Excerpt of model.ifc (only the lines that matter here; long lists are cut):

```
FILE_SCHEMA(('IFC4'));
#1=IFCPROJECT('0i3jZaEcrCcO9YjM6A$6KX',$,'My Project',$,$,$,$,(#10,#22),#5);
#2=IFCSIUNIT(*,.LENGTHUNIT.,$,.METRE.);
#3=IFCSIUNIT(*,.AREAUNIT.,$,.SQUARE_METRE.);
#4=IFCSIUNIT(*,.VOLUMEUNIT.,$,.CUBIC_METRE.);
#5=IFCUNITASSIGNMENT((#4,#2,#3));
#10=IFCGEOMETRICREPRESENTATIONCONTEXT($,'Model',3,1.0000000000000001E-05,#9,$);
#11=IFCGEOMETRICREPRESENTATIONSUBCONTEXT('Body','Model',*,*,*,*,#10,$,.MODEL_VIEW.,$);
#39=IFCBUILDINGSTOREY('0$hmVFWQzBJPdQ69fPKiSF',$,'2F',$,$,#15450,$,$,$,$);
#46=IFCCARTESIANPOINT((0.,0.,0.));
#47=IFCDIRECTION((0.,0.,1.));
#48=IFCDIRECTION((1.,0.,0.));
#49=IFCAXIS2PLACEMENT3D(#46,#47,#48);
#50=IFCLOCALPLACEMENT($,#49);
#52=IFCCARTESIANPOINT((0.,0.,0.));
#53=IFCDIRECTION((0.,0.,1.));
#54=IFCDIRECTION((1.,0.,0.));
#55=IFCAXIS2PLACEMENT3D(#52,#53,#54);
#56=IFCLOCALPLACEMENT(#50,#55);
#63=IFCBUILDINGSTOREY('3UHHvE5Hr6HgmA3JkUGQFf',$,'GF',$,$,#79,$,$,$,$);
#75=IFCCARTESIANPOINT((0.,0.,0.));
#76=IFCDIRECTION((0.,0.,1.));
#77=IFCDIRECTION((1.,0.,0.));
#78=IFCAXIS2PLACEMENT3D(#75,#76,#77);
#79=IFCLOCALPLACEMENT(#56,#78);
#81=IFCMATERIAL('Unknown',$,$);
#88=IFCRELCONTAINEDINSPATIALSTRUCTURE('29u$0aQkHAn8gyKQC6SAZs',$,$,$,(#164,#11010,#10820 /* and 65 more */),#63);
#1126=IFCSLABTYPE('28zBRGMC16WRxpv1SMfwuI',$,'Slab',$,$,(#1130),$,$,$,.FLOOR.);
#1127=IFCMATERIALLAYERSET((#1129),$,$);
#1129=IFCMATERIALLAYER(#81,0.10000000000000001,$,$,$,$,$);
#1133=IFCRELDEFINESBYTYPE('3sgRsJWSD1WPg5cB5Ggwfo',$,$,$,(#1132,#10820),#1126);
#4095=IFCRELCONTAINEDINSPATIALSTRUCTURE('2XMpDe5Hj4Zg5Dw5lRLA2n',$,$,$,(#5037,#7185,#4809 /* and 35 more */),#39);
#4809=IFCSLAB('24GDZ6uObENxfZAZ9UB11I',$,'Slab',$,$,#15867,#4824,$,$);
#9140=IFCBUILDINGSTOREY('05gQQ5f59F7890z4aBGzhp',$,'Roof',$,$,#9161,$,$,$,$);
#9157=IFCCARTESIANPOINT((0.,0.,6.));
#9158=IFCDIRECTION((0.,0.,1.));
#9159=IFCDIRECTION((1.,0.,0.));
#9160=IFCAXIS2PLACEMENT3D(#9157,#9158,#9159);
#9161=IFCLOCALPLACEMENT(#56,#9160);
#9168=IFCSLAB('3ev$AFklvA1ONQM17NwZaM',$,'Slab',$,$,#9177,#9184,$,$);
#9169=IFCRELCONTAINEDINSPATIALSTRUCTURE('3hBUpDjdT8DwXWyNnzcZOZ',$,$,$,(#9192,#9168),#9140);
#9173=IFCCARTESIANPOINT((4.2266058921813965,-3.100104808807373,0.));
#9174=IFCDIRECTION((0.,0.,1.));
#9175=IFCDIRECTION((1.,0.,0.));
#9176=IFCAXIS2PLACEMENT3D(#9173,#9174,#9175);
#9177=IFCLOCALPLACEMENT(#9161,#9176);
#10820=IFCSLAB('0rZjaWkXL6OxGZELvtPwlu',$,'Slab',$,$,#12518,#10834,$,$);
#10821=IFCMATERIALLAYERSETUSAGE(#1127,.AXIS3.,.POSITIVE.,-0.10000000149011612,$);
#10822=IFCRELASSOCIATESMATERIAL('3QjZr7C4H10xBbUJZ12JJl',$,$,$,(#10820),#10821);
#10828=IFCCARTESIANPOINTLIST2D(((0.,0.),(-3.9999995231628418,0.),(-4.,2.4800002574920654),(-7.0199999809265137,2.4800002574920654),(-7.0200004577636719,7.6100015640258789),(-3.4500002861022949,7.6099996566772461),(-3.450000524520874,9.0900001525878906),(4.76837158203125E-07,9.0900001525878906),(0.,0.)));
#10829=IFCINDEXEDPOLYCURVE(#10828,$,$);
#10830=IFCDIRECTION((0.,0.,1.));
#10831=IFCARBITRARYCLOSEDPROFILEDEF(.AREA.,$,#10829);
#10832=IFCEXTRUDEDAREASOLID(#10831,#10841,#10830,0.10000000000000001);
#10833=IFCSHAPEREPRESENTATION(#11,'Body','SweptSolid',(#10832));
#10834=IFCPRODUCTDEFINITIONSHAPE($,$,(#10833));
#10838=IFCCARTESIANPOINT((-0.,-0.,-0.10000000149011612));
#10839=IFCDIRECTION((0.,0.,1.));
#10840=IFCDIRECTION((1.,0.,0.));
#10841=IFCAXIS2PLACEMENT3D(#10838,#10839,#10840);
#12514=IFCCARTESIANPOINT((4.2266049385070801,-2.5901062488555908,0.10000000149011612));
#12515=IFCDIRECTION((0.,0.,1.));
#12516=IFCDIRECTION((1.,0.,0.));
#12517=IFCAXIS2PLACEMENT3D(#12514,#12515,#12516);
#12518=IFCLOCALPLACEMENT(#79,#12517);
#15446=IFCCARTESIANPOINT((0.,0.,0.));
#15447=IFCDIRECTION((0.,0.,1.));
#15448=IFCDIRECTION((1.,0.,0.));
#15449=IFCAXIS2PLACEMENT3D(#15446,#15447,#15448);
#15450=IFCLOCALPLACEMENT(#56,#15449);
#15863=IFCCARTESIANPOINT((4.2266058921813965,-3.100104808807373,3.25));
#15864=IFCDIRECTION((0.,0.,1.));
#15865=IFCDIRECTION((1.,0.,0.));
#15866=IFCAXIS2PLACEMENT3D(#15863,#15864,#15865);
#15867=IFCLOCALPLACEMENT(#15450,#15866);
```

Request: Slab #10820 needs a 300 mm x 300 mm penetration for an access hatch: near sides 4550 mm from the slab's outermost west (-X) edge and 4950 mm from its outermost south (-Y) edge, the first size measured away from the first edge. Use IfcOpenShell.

```python
import numpy as np
import ifcopenshell
import ifcopenshell.api.feature
import ifcopenshell.api.geometry
import ifcopenshell.api.root
import ifcopenshell.geom
import ifcopenshell.util.placement
import ifcopenshell.util.representation
import ifcopenshell.util.shape
import ifcopenshell.util.unit

model = ifcopenshell.open("model.ifc")
unit_scale = ifcopenshell.util.unit.calculate_unit_scale(model)
settings = ifcopenshell.geom.settings()


def volume(element):
    """Net volume in cubic metres, openings subtracted."""
    shape = ifcopenshell.geom.create_shape(settings, element)
    return ifcopenshell.util.shape.get_volume(shape.geometry)


slab = model.by_id(10820)
before = volume(slab)

# Extent in the slab's own axes, in metres. The edges named are its -X and -Y sides.
slab_shape = ifcopenshell.geom.create_shape(settings, slab)
vertices = ifcopenshell.util.shape.get_vertices(slab_shape.geometry)
x_min, y_min, bottom = vertices.min(axis=0)
top = vertices[:, 2].max()

opening = ifcopenshell.api.root.create_entity(model, ifc_class="IfcOpeningElement", name="Access hatch opening", predefined_type="OPENING")
context = ifcopenshell.util.representation.get_context(model, "Model", "Body", "MODEL_VIEW")
width, depth = 0.3, 0.3
outline = [(0.0, 0.0), (width, 0.0), (width, depth), (0.0, depth), (0.0, 0.0)]
# Overshoot both faces by 50 mm so the cut is clean.
shape = ifcopenshell.api.geometry.add_slab_representation(
    model, context=context, depth=top - bottom + 0.1, polyline=outline
)
ifcopenshell.api.geometry.assign_representation(model, product=opening, representation=shape)

matrix = ifcopenshell.util.placement.get_local_placement(slab.ObjectPlacement)
matrix[:, 3] = matrix @ np.append(np.array([x_min + 4.55, y_min + 4.95, bottom - 0.05]) / unit_scale, 1.0)
ifcopenshell.api.geometry.edit_object_placement(model, product=opening, matrix=matrix, is_si=False)
ifcopenshell.api.feature.add_feature(model, feature=opening, element=slab)

after = volume(slab)

print(f"slab volume {before:.3f} -> {after:.3f} m3")

model.write("model_rev.ifc")
```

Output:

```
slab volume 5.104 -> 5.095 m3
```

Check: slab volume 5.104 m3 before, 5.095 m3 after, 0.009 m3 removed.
